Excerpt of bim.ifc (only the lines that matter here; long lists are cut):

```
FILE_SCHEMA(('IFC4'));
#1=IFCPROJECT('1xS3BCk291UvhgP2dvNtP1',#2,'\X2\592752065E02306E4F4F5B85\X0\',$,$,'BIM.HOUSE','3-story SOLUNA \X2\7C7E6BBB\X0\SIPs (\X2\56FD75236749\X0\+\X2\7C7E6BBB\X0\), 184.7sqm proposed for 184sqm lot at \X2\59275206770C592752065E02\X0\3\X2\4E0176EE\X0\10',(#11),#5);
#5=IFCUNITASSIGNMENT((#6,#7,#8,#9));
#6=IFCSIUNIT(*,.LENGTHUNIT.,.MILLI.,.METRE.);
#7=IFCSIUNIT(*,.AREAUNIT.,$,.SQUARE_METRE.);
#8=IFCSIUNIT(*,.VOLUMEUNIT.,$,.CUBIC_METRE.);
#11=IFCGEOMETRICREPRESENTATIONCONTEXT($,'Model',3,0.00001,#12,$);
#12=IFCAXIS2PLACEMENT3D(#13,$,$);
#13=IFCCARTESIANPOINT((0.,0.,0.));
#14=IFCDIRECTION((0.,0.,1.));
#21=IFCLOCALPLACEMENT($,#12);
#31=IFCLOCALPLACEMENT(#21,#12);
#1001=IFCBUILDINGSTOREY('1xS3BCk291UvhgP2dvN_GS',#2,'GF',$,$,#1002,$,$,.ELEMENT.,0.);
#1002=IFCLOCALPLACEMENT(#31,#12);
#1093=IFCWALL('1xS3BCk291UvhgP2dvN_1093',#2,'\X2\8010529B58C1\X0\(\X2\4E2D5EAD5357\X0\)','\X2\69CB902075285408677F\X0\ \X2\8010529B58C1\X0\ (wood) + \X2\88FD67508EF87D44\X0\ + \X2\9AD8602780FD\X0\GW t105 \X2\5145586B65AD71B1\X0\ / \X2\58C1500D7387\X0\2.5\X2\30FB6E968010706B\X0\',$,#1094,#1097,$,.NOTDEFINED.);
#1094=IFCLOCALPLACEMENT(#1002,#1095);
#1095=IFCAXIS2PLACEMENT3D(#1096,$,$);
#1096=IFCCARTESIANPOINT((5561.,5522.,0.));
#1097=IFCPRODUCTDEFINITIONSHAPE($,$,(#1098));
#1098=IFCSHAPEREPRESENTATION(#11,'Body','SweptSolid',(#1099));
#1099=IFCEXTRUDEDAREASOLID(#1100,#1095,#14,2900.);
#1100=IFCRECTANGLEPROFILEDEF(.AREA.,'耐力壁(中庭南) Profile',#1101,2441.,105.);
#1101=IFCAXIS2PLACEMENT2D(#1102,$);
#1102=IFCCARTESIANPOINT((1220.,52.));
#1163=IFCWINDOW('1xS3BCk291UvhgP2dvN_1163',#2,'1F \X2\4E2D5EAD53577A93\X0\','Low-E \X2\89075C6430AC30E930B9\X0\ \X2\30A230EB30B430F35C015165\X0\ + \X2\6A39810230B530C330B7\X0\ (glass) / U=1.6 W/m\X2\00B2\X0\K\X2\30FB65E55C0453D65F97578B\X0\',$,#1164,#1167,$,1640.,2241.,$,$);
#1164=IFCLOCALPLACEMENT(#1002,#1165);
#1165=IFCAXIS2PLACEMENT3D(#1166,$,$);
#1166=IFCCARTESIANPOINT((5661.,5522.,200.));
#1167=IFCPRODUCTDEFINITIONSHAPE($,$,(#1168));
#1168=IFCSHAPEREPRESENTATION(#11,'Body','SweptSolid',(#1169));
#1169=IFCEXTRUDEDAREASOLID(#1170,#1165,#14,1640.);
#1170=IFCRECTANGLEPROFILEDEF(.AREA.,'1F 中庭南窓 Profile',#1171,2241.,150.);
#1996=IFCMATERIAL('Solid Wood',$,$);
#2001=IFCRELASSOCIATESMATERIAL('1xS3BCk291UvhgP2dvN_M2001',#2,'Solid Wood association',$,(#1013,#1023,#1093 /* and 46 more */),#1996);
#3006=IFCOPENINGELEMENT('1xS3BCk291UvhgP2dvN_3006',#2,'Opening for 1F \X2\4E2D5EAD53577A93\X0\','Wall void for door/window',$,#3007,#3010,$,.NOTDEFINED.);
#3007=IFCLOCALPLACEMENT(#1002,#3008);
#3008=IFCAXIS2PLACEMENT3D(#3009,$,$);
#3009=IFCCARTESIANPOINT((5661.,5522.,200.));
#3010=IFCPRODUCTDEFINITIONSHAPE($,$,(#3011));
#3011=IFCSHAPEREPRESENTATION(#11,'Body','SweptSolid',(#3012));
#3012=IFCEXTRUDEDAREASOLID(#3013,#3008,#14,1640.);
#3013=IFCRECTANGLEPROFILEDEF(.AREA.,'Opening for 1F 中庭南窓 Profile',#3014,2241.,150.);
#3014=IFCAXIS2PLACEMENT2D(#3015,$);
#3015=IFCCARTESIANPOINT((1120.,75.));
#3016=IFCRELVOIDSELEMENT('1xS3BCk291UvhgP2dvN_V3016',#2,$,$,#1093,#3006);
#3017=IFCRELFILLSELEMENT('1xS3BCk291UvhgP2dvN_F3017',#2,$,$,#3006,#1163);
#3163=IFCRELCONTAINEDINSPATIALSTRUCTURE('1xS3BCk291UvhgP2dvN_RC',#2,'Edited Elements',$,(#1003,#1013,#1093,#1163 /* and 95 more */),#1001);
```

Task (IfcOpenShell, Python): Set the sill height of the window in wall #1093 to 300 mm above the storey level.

```python
import numpy as np
import ifcopenshell
import ifcopenshell.api.geometry
import ifcopenshell.geom
import ifcopenshell.util.element
import ifcopenshell.util.placement
import ifcopenshell.util.shape
import ifcopenshell.util.unit

model = ifcopenshell.open("bim.ifc")
unit_scale = ifcopenshell.util.unit.calculate_unit_scale(model)

window = model.by_guid("1xS3BCk291UvhgP2dvN_1163")
opening = window.FillsVoids[0].RelatingOpeningElement
storey = ifcopenshell.util.element.get_container(window, ifc_class="IfcBuildingStorey")
level = ifcopenshell.util.placement.get_local_placement(storey.ObjectPlacement)[2, 3]

# The opening's origin need not be at the sill, so measure its lowest point.
shape = ifcopenshell.geom.create_shape(ifcopenshell.geom.settings(), opening)
bottom = ifcopenshell.util.shape.get_shape_bottom_elevation(shape, shape.geometry) / unit_scale
dz = level + 0.3 / unit_scale - bottom

shift = np.array([0.0, 0.0, dz])
# The window is not placed relative to its opening, so move both.
for product in (opening, window):
    matrix = ifcopenshell.util.placement.get_local_placement(product.ObjectPlacement)
    matrix[:3, 3] += shift
    ifcopenshell.api.geometry.edit_object_placement(model, product=product, matrix=matrix, is_si=False)

print(f"moved by {dz * unit_scale:+.3f} m")

model.write("bim_v2.ifc")
```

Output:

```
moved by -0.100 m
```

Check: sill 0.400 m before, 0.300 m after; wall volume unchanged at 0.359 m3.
